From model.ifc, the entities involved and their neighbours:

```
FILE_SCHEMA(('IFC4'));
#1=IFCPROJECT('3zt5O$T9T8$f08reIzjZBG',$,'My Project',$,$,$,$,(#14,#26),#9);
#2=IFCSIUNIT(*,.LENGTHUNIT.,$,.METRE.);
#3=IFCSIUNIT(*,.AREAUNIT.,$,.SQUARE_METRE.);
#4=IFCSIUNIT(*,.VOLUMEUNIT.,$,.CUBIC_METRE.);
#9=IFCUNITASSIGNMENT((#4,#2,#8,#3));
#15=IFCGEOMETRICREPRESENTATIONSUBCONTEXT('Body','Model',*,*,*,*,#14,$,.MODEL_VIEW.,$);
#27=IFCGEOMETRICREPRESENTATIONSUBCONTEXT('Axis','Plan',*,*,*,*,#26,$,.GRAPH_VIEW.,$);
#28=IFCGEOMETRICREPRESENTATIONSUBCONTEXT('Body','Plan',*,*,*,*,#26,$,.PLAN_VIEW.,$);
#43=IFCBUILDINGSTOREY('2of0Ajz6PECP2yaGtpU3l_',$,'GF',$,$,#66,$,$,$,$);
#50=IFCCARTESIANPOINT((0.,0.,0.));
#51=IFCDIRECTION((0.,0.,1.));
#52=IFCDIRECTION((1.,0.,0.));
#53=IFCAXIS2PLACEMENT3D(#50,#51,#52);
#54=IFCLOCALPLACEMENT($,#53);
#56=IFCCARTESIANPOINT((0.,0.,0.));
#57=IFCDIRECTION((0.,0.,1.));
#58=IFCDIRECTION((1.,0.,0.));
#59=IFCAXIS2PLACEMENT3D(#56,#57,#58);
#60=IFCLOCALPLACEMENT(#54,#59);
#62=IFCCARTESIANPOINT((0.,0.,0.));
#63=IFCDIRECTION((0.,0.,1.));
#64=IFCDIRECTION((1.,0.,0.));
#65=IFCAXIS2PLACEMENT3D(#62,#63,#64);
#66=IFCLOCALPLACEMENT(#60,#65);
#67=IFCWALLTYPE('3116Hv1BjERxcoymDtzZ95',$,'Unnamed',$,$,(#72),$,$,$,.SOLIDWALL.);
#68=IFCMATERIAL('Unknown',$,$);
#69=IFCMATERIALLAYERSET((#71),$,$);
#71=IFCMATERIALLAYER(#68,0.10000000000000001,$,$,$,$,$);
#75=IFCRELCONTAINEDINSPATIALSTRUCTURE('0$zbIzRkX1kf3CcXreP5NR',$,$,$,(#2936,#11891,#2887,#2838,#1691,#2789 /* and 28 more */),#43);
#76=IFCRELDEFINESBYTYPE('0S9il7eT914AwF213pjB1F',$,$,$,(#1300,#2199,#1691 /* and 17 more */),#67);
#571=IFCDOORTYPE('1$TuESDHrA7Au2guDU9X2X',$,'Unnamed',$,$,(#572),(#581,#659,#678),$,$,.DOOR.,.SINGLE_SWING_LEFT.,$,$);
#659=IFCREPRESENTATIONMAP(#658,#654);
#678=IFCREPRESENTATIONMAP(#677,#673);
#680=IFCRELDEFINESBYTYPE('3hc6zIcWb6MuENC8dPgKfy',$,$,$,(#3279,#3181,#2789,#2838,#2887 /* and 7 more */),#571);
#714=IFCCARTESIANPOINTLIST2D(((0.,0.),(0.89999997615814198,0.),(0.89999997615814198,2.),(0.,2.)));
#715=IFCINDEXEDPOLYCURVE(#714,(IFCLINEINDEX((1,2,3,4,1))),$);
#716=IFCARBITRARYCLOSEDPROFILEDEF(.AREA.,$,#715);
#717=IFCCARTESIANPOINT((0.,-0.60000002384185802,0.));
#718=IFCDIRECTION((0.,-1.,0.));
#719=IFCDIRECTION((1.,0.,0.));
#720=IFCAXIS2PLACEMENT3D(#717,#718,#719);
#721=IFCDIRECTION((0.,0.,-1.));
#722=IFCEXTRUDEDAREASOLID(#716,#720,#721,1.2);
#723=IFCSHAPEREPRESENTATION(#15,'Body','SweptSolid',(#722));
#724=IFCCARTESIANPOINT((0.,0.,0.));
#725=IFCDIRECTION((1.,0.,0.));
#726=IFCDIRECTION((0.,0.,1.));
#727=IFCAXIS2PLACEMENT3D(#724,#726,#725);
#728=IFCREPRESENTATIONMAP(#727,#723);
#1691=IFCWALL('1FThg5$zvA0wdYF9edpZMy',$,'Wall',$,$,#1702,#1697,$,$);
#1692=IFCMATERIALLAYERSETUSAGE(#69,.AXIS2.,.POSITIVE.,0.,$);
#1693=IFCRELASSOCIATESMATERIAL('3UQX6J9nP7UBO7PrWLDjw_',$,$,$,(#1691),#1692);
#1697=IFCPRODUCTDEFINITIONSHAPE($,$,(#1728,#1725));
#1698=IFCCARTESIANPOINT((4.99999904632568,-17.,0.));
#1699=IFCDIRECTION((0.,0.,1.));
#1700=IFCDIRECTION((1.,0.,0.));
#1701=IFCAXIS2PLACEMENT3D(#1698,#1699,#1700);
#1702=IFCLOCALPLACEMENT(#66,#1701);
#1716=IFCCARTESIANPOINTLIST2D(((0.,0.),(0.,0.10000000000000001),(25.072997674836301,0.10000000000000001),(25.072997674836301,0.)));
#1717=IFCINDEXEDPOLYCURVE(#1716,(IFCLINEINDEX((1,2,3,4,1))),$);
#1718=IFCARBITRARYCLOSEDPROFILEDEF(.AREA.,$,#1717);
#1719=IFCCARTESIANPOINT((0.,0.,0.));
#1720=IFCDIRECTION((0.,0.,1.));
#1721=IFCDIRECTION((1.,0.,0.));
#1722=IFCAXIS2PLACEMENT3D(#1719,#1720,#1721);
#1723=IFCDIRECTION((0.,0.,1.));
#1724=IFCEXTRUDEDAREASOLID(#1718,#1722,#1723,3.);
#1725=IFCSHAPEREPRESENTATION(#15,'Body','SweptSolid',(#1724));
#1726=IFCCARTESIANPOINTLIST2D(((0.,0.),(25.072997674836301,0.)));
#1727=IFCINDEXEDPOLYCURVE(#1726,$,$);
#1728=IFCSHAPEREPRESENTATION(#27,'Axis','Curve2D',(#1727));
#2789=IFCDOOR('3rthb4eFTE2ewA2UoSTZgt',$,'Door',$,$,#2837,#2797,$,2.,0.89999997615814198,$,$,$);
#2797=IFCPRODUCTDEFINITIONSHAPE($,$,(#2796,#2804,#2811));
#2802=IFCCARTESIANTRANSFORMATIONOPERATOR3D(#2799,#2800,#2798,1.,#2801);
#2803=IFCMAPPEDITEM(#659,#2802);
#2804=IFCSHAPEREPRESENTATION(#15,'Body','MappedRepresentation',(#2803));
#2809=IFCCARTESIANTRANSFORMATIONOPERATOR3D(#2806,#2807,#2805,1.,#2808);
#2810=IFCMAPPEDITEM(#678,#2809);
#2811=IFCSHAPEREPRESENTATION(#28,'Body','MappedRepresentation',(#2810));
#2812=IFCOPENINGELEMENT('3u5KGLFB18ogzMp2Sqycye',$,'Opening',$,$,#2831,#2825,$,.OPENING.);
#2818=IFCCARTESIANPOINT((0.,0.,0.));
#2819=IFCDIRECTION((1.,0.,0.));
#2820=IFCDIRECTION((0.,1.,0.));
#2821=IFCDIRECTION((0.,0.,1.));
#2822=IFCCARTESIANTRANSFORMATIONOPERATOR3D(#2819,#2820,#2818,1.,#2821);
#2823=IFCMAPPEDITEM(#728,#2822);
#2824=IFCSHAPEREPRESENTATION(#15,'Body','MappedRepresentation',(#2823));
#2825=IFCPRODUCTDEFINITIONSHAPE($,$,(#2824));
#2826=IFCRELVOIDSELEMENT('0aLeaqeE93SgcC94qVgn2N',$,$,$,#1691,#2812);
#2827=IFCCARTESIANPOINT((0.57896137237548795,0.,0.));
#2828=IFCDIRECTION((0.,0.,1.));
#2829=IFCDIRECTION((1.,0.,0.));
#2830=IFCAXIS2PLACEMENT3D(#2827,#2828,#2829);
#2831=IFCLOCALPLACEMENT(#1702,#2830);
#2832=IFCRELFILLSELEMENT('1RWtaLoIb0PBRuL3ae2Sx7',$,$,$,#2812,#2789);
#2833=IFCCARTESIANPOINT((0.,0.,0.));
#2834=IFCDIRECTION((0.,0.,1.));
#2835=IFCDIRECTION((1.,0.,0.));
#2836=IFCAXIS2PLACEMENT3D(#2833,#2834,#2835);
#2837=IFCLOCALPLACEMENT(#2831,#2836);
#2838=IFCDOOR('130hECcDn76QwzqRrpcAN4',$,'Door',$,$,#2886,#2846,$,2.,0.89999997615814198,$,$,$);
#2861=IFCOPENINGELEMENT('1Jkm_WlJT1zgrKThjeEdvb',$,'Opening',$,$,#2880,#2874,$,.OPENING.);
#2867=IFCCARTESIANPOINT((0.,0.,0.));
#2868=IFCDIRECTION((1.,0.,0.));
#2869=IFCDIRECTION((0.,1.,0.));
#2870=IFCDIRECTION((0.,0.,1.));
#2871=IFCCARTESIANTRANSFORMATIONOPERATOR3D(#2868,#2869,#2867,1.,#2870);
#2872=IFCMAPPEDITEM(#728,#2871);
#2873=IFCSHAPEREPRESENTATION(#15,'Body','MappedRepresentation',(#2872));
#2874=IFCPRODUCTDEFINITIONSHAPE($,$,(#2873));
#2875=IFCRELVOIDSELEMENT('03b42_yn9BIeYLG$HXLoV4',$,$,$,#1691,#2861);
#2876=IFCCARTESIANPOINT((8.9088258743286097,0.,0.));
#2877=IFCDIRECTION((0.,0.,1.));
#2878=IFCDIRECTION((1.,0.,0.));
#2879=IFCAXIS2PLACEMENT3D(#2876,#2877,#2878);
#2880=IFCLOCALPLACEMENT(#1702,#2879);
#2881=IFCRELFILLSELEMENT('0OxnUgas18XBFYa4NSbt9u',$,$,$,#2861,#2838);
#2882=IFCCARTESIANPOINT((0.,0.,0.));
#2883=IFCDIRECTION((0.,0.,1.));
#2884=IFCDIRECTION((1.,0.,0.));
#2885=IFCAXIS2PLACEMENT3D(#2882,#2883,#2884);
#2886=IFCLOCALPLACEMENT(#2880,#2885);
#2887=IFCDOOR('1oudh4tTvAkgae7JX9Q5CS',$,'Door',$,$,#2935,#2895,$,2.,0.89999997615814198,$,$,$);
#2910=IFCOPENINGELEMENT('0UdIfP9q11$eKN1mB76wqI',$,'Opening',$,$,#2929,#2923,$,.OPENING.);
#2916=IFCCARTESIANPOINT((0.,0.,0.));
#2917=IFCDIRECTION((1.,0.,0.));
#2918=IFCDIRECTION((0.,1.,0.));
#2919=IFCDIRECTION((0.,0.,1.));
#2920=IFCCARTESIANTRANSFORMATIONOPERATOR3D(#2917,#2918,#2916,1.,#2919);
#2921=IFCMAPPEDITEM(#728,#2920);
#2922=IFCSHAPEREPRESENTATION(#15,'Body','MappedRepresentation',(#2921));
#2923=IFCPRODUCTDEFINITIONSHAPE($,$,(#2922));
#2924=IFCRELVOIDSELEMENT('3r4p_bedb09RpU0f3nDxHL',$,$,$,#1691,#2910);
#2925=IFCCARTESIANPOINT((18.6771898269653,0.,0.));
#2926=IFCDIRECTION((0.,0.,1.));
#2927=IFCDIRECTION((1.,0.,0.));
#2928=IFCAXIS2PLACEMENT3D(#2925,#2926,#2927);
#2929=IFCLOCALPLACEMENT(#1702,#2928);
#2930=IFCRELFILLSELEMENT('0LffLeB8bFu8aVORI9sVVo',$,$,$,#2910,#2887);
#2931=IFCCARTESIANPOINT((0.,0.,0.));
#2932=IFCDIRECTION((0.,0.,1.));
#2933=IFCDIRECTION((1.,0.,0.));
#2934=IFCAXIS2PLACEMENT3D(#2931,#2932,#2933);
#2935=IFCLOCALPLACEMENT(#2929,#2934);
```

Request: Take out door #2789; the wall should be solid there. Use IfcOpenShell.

```python
import ifcopenshell
import ifcopenshell.api.feature
import ifcopenshell.api.root
import ifcopenshell.geom
import ifcopenshell.util.shape

model = ifcopenshell.open("model.ifc")
settings = ifcopenshell.geom.settings()


def volume(element):
    """Net volume in cubic metres, openings subtracted."""
    shape = ifcopenshell.geom.create_shape(settings, element)
    return ifcopenshell.util.shape.get_volume(shape.geometry)


door = model.by_guid("3rthb4eFTE2ewA2UoSTZgt")
opening = door.FillsVoids[0].RelatingOpeningElement
wall = opening.VoidsElements[0].RelatingBuildingElement
before = volume(wall)

ifcopenshell.api.root.remove_product(model, product=door)
ifcopenshell.api.feature.remove_feature(model, feature=opening)

after = volume(wall)

print(f"wall volume {before:.3f} -> {after:.3f} m3")

model.write("model_updated.ifc")
```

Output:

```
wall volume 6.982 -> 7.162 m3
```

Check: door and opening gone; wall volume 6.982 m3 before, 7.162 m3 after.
